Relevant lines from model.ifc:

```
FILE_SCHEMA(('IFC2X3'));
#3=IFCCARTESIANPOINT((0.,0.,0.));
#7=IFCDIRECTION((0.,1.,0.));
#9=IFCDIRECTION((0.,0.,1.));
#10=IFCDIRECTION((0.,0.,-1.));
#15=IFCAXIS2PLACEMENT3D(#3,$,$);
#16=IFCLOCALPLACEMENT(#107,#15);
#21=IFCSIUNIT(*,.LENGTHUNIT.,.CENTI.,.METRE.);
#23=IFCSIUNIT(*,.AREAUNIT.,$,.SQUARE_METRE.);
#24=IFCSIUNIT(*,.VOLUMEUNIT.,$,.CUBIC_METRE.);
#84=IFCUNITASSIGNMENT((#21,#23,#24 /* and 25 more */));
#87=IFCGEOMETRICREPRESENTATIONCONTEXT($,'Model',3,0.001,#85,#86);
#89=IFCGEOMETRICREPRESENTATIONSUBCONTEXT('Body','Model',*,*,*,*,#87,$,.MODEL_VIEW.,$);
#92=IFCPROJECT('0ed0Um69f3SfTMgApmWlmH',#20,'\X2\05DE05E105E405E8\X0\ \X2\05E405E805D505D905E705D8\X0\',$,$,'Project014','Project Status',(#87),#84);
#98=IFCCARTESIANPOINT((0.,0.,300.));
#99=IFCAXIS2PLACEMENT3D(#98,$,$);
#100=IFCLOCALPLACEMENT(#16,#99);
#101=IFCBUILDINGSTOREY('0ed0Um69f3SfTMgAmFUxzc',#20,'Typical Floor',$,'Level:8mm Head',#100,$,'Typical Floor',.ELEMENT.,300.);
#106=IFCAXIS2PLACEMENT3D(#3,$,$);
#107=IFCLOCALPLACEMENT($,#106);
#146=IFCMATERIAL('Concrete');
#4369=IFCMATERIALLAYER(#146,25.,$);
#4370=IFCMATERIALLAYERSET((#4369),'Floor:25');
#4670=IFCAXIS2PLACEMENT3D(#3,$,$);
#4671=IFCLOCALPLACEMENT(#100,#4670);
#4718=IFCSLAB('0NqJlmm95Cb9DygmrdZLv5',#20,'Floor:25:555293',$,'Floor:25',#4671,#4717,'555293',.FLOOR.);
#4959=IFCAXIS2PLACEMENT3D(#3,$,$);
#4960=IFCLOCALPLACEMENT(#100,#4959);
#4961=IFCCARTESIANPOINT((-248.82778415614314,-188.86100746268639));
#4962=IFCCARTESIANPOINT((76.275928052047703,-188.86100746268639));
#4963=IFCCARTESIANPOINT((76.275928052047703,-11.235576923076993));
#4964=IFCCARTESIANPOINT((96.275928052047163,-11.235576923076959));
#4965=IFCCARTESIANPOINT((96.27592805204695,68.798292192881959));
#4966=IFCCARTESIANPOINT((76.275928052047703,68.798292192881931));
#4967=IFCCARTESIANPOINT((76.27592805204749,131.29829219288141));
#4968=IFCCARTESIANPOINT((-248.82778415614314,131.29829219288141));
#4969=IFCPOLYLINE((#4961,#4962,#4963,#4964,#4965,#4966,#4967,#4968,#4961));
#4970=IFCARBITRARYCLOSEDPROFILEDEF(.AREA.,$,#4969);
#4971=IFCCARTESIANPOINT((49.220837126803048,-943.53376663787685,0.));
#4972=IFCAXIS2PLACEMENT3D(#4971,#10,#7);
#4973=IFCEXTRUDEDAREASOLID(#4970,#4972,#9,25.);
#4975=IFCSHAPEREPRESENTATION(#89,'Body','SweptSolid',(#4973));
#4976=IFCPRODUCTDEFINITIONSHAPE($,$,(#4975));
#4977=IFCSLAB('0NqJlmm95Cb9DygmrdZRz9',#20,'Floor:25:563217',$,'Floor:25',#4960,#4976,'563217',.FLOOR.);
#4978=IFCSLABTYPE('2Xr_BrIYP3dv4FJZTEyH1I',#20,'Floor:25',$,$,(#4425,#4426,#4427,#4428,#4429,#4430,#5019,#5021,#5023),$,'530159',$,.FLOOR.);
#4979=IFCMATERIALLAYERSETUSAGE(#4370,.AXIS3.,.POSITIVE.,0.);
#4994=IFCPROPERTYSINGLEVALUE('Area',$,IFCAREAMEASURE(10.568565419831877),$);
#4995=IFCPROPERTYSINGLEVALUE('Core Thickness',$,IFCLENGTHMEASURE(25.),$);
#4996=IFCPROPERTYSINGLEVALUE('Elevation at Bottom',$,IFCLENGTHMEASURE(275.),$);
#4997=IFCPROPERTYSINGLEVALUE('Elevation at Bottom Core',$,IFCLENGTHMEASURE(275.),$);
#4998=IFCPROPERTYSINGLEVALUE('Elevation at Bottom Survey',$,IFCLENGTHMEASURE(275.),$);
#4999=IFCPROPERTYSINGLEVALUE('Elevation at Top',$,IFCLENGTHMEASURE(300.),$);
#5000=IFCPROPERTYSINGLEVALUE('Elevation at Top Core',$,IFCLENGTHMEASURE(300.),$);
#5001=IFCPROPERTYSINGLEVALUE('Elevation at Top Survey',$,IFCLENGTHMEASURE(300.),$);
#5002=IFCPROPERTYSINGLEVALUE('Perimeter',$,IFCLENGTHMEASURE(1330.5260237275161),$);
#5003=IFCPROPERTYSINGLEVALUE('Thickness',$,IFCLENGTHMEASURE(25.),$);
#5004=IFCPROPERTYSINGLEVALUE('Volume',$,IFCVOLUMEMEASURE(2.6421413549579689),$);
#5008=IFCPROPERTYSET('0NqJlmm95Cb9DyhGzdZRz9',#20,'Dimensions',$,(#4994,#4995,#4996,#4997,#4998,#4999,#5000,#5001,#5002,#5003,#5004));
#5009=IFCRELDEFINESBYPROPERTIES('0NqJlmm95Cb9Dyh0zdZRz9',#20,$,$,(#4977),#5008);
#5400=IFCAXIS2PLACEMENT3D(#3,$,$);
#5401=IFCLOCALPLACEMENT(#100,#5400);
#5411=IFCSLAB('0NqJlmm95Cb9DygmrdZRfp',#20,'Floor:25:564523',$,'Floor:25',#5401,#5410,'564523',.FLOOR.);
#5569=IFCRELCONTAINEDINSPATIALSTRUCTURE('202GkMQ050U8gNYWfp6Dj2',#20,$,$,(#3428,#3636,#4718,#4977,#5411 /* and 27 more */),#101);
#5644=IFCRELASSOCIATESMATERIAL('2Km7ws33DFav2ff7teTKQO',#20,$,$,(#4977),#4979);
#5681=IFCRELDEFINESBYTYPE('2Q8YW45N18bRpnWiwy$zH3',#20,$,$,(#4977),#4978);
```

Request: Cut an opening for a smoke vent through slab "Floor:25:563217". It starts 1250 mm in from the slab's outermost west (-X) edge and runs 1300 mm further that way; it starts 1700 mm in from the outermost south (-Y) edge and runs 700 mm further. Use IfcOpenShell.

```python
import numpy as np
import ifcopenshell
import ifcopenshell.api.feature
import ifcopenshell.api.geometry
import ifcopenshell.api.pset
import ifcopenshell.api.root
import ifcopenshell.geom
import ifcopenshell.util.element
import ifcopenshell.util.placement
import ifcopenshell.util.representation
import ifcopenshell.util.shape
import ifcopenshell.util.unit

model = ifcopenshell.open("model.ifc")
unit_scale = ifcopenshell.util.unit.calculate_unit_scale(model)
area_scale = ifcopenshell.util.unit.calculate_unit_scale(model, "AREAUNIT")
volume_scale = ifcopenshell.util.unit.calculate_unit_scale(model, "VOLUMEUNIT")
settings = ifcopenshell.geom.settings()


def volume(element):
    """Net volume in cubic metres, openings subtracted."""
    shape = ifcopenshell.geom.create_shape(settings, element)
    return ifcopenshell.util.shape.get_volume(shape.geometry)


slab = model.by_guid("0NqJlmm95Cb9DygmrdZRz9")
before = volume(slab)

# Extent in the slab's own axes, in metres. The edges named are its -X and -Y sides.
slab_shape = ifcopenshell.geom.create_shape(settings, slab)
vertices = ifcopenshell.util.shape.get_vertices(slab_shape.geometry)
x_min, y_min, bottom = vertices.min(axis=0)
top = vertices[:, 2].max()

opening = ifcopenshell.api.root.create_entity(model, ifc_class="IfcOpeningElement", name="Smoke vent opening")
context = ifcopenshell.util.representation.get_context(model, "Model", "Body", "MODEL_VIEW")
width, depth = 1.3, 0.7
outline = [(0.0, 0.0), (width, 0.0), (width, depth), (0.0, depth), (0.0, 0.0)]
# Overshoot both faces by 50 mm so the cut is clean.
shape = ifcopenshell.api.geometry.add_slab_representation(
    model, context=context, depth=top - bottom + 0.1, polyline=outline
)
ifcopenshell.api.geometry.assign_representation(model, product=opening, representation=shape)

matrix = ifcopenshell.util.placement.get_local_placement(slab.ObjectPlacement)
matrix[:, 3] = matrix @ np.append(np.array([x_min + 1.25, y_min + 1.7, bottom - 0.05]) / unit_scale, 1.0)
ifcopenshell.api.geometry.edit_object_placement(model, product=opening, matrix=matrix, is_si=False)
ifcopenshell.api.feature.add_feature(model, feature=opening, element=slab)

after = volume(slab)

# Update the slab's stored quantities.
pset = model.by_id(ifcopenshell.util.element.get_pset(slab, "Dimensions", should_inherit=False)["id"])
ifcopenshell.api.pset.edit_pset(model, pset=pset, properties={
    "Area": model.create_entity("IfcAreaMeasure", after / (top - bottom) / area_scale),
    "Volume": model.create_entity("IfcVolumeMeasure", after / volume_scale),
})

print(f"slab volume {before:.3f} -> {after:.3f} m3")

model.write("model_edited.ifc")
```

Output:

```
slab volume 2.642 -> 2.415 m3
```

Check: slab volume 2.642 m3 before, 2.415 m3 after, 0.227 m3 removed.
